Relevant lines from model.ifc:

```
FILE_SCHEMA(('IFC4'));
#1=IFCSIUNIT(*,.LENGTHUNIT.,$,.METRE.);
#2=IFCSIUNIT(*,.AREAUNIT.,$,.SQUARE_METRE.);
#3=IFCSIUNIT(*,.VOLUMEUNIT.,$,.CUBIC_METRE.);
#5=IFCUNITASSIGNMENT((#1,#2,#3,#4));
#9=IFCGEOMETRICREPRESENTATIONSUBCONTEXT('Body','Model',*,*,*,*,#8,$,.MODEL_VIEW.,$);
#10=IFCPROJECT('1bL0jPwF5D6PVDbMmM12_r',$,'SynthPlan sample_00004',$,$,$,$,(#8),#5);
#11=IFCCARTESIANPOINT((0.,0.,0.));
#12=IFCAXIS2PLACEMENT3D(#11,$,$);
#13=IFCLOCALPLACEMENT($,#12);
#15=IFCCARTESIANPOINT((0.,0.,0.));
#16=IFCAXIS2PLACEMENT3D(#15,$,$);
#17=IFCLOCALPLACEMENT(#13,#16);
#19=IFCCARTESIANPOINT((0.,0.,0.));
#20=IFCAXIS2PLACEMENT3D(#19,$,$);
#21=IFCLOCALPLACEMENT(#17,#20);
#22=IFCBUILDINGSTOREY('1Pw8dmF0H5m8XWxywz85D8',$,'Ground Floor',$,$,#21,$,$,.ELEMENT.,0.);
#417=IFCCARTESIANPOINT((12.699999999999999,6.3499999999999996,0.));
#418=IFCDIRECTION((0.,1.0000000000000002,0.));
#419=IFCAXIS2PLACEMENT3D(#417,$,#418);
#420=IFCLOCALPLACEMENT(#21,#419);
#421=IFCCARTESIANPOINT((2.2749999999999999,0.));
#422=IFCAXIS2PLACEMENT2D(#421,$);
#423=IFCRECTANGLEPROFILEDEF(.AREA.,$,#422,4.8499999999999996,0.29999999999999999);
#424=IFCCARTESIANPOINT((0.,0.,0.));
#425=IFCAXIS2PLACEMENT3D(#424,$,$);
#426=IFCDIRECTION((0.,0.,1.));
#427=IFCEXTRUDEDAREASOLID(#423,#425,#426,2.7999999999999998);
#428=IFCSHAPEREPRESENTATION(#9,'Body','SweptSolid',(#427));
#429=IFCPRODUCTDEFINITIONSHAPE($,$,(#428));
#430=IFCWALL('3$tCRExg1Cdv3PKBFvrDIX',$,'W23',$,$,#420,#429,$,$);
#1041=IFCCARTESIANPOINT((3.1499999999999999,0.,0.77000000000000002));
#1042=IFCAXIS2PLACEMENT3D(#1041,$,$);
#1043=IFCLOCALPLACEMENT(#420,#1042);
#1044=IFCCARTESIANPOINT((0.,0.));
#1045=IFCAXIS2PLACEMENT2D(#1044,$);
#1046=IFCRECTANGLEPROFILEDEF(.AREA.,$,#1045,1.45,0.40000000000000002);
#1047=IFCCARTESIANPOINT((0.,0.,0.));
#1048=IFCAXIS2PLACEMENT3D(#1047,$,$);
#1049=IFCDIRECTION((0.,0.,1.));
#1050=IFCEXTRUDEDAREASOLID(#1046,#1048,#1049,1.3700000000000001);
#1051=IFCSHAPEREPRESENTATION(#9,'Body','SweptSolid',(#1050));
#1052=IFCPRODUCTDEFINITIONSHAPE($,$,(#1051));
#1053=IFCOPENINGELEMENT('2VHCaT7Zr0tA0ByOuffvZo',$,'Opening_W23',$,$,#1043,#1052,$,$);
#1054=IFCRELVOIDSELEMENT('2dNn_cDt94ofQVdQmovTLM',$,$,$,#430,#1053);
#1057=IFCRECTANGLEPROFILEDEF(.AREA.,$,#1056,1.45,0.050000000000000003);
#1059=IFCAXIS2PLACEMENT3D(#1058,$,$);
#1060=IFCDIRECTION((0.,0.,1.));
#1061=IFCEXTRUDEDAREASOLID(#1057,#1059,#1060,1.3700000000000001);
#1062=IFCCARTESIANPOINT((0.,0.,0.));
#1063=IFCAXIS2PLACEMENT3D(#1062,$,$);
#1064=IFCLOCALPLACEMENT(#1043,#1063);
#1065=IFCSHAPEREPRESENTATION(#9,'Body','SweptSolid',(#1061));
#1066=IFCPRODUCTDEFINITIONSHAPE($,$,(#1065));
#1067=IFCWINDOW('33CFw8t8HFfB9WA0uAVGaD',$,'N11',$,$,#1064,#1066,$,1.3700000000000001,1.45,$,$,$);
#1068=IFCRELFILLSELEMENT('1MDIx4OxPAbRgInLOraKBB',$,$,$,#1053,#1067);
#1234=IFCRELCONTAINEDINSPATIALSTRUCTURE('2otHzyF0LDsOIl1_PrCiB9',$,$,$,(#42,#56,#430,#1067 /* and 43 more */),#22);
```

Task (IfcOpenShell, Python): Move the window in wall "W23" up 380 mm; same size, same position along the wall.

```python
import numpy as np
import ifcopenshell
import ifcopenshell.api.geometry
import ifcopenshell.util.placement
import ifcopenshell.util.unit

model = ifcopenshell.open("model.ifc")
unit_scale = ifcopenshell.util.unit.calculate_unit_scale(model)

window = model.by_guid("33CFw8t8HFfB9WA0uAVGaD")
opening = window.FillsVoids[0].RelatingOpeningElement
dz = 0.38 / unit_scale

shift = np.array([0.0, 0.0, dz])
# The window is placed relative to its opening, so it follows when the opening moves.
matrix = ifcopenshell.util.placement.get_local_placement(opening.ObjectPlacement)
matrix[:3, 3] += shift
ifcopenshell.api.geometry.edit_object_placement(
    model, product=opening, matrix=matrix, is_si=False, should_transform_children=True
)

print(f"moved by {dz * unit_scale:+.3f} m")

model.write("model_edited.ifc")
```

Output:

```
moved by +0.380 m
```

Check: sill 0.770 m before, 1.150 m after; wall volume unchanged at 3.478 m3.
